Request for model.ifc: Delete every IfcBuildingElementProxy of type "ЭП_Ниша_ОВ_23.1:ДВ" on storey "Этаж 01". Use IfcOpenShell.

First a look at what the model holds.

```python
import ifcopenshell
import ifcopenshell.util.element

model = ifcopenshell.open("model.ifc")
print(model.schema)
storey = next(s for s in model.by_type("IfcBuildingStorey") if s.Name == "Этаж 01")
proxies = [e for e in ifcopenshell.util.element.get_decomposition(storey) if e.is_a("IfcBuildingElementProxy")]
seen = {}
for e in proxies:
    element_type = ifcopenshell.util.element.get_type(e)
    name = element_type.Name if element_type not in (None, e) else None
    seen[name] = seen.get(name, 0) + 1
for name, count in sorted(seen.items(), key=str):
    print(count, "x", name)
```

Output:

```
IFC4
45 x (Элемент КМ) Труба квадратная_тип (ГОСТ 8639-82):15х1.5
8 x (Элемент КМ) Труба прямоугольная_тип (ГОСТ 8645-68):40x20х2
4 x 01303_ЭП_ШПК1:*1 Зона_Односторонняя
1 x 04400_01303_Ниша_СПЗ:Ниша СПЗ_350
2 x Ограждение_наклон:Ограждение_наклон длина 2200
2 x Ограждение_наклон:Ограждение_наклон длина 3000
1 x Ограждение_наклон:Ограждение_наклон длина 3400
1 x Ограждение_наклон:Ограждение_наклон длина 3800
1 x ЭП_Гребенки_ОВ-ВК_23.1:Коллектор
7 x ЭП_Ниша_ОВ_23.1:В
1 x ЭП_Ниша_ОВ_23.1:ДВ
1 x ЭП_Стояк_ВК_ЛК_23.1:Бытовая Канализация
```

```python
import ifcopenshell
import ifcopenshell.api.root
import ifcopenshell.util.element

model = ifcopenshell.open("model.ifc")

storey = next(s for s in model.by_type("IfcBuildingStorey") if s.Name == "Этаж 01")
proxies = [e for e in ifcopenshell.util.element.get_decomposition(storey) if e.is_a("IfcBuildingElementProxy")]
targets = [e for e in proxies if (t := ifcopenshell.util.element.get_type(e)) not in (None, e) and t.Name == "ЭП_Ниша_ОВ_23.1:ДВ"]

for e in targets:
    ifcopenshell.api.root.remove_product(model, product=e)
print(len(targets), "removed")

model.write("model_edited.ifc")
```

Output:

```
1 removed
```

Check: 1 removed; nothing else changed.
